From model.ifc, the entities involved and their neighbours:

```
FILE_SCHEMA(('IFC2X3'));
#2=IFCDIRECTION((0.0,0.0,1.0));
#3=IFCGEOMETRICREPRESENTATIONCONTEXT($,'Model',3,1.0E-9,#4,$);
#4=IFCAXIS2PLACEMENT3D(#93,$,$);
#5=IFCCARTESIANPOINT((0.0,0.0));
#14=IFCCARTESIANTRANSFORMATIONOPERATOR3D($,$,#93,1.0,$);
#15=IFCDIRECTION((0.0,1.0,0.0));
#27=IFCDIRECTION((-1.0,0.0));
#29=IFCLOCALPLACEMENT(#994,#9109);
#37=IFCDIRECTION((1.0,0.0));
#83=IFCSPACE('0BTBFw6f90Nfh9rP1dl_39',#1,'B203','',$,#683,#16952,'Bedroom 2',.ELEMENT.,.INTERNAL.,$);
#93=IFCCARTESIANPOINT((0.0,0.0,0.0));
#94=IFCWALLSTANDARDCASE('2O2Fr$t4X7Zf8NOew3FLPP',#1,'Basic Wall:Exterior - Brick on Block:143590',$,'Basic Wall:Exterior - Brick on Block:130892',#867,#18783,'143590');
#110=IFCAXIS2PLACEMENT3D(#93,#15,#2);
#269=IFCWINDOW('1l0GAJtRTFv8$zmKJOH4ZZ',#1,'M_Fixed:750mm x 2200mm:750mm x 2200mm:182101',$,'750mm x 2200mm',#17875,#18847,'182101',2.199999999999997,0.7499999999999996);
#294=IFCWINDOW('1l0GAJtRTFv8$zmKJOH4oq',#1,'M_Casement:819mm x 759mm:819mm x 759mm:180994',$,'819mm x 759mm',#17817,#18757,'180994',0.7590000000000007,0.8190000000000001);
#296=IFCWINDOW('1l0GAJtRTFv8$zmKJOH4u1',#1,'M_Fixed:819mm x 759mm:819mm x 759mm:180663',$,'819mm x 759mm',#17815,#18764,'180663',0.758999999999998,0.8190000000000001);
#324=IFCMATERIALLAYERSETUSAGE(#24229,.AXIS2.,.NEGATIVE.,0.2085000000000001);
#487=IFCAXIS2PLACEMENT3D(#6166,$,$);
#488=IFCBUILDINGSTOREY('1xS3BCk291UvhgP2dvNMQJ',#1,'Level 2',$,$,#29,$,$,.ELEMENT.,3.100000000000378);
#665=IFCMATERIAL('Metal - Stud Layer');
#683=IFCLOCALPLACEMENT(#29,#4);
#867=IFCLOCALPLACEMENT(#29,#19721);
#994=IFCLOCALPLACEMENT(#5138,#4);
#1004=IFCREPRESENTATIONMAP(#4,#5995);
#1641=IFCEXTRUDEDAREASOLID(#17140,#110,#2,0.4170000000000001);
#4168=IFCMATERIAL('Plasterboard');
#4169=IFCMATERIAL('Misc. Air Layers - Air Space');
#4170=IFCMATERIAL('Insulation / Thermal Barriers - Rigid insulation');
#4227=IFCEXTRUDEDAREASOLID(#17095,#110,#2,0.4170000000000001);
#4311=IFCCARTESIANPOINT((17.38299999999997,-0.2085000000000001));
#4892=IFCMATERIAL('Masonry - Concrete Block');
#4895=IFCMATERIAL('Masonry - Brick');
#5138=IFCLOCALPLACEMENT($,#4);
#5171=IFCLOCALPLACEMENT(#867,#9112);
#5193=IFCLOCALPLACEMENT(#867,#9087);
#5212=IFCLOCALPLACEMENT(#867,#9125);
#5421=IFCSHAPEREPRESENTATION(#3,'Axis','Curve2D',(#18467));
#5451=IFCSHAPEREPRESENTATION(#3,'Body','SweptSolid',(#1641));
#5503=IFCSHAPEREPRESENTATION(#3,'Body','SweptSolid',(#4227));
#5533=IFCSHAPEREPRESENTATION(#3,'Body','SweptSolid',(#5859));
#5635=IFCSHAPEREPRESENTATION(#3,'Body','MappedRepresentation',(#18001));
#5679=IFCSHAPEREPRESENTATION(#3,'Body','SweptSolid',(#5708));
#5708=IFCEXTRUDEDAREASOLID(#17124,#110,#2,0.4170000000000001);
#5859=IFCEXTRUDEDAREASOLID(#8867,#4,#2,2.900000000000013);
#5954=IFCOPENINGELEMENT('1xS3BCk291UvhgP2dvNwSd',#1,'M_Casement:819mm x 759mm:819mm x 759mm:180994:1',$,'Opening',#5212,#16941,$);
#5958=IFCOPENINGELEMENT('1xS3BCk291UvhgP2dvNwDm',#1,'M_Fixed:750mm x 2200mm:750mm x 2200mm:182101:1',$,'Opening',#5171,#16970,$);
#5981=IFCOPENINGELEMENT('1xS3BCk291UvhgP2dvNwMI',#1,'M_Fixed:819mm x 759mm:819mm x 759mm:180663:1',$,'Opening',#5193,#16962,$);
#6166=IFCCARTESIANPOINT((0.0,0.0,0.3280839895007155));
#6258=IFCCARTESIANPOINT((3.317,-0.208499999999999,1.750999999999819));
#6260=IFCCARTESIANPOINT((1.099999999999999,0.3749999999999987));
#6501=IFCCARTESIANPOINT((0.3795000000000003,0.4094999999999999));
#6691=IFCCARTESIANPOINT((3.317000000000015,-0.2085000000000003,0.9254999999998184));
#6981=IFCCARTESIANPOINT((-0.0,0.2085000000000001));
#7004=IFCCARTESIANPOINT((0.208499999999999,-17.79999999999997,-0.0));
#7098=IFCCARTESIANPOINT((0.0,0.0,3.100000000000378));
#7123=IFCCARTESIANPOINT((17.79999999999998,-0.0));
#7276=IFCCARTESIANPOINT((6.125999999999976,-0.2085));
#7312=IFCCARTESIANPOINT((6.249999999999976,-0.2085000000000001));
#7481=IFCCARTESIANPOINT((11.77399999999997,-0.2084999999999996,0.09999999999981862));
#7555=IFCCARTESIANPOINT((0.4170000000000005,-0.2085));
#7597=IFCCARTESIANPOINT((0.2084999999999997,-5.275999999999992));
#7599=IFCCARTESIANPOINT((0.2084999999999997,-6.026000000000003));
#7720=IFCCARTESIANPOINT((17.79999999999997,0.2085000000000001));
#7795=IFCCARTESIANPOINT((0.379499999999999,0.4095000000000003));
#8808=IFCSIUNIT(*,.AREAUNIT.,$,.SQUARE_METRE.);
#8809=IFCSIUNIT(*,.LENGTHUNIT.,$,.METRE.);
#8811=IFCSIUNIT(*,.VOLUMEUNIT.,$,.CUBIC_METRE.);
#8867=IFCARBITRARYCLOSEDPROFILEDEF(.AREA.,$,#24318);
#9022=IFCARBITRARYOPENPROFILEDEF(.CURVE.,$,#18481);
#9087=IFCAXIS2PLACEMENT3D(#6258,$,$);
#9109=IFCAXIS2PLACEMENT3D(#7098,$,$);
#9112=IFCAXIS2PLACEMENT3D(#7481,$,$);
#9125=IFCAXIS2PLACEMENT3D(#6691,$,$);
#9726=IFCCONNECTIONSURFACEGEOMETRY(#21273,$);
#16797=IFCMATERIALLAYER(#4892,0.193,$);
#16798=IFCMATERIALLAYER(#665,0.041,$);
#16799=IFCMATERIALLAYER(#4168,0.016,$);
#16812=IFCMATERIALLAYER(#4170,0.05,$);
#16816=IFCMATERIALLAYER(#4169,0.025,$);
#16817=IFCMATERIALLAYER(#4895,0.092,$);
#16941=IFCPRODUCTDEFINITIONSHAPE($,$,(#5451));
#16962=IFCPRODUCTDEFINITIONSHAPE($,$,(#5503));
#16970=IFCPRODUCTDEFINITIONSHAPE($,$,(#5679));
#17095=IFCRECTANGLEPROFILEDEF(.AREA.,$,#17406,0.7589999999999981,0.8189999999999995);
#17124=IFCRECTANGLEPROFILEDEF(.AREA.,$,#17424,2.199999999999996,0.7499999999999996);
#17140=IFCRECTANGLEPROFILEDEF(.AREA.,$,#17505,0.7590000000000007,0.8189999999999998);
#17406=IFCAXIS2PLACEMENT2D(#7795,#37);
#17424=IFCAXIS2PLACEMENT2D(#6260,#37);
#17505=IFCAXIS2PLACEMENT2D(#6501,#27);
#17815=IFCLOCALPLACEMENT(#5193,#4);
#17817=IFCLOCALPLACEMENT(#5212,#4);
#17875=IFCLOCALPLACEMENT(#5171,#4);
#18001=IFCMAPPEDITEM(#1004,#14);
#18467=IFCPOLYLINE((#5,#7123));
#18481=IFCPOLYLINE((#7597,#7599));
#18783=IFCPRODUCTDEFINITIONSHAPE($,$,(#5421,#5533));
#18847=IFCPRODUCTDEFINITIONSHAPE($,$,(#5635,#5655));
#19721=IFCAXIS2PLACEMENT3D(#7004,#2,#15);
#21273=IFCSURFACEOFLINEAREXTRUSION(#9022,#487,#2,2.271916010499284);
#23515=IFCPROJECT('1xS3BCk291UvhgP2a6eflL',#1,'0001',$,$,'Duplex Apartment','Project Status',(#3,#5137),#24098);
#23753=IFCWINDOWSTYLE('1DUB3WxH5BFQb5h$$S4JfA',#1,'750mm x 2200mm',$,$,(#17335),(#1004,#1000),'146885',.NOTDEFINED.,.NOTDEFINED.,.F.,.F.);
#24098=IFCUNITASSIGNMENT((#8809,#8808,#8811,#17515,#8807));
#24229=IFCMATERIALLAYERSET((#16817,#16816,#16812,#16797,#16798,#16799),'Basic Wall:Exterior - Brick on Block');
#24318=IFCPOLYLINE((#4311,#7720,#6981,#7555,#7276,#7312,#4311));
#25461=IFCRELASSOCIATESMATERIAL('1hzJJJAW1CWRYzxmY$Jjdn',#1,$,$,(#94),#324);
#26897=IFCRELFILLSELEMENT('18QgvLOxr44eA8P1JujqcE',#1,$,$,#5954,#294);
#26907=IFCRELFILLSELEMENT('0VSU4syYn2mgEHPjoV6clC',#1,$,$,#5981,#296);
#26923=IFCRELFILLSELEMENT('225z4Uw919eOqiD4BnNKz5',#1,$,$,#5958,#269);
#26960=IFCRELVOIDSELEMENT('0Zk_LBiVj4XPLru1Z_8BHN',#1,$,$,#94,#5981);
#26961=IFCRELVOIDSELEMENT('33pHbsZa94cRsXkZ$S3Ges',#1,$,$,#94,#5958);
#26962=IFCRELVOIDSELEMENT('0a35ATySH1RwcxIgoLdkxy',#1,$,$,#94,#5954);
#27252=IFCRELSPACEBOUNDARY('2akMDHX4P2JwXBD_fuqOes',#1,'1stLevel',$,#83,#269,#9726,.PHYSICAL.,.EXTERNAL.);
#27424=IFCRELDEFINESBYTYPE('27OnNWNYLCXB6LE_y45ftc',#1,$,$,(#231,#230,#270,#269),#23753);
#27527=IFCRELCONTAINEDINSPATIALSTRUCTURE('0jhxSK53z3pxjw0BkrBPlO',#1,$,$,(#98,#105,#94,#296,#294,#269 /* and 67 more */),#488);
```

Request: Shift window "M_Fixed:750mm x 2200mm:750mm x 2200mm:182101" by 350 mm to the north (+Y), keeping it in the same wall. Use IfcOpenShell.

```python
import numpy as np
import ifcopenshell
import ifcopenshell.api.geometry
import ifcopenshell.util.placement

model = ifcopenshell.open("model.ifc")

window = model.by_guid("1l0GAJtRTFv8$zmKJOH4ZZ")
opening = window.FillsVoids[0].RelatingOpeningElement
wall = opening.VoidsElements[0].RelatingBuildingElement

wall_matrix = ifcopenshell.util.placement.get_local_placement(wall.ObjectPlacement)
shift = wall_matrix[:3, 0] * 0.35
before = ifcopenshell.util.placement.get_local_placement(window.ObjectPlacement)[:3, 3].copy()

# The window is placed relative to its opening, so it follows when the opening moves.
matrix = ifcopenshell.util.placement.get_local_placement(opening.ObjectPlacement)
matrix[:3, 3] += shift
ifcopenshell.api.geometry.edit_object_placement(
    model, product=opening, matrix=matrix, is_si=False, should_transform_children=True
)

# Space boundary surfaces are stored in each space's coordinates; move them too.
for rel in window.ProvidesBoundaries:
    if not rel.ConnectionGeometry:
        continue
    surface = rel.ConnectionGeometry.SurfaceOnRelatingElement
    space_matrix = ifcopenshell.util.placement.get_local_placement(rel.RelatingSpace.ObjectPlacement)
    point = np.array(surface.Position.Location.Coordinates) + space_matrix[:3, :3].T @ shift
    surface.Position = model.createIfcAxis2Placement3D(
        model.createIfcCartesianPoint(point.tolist()), surface.Position.Axis, surface.Position.RefDirection
    )

after = ifcopenshell.util.placement.get_local_placement(window.ObjectPlacement)[:3, 3]
print("window moved by", (after - before).round(3) + 0.0)

model.write("model_rev.ifc")
```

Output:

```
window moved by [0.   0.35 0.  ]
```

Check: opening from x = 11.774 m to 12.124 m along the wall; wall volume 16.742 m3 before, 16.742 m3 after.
